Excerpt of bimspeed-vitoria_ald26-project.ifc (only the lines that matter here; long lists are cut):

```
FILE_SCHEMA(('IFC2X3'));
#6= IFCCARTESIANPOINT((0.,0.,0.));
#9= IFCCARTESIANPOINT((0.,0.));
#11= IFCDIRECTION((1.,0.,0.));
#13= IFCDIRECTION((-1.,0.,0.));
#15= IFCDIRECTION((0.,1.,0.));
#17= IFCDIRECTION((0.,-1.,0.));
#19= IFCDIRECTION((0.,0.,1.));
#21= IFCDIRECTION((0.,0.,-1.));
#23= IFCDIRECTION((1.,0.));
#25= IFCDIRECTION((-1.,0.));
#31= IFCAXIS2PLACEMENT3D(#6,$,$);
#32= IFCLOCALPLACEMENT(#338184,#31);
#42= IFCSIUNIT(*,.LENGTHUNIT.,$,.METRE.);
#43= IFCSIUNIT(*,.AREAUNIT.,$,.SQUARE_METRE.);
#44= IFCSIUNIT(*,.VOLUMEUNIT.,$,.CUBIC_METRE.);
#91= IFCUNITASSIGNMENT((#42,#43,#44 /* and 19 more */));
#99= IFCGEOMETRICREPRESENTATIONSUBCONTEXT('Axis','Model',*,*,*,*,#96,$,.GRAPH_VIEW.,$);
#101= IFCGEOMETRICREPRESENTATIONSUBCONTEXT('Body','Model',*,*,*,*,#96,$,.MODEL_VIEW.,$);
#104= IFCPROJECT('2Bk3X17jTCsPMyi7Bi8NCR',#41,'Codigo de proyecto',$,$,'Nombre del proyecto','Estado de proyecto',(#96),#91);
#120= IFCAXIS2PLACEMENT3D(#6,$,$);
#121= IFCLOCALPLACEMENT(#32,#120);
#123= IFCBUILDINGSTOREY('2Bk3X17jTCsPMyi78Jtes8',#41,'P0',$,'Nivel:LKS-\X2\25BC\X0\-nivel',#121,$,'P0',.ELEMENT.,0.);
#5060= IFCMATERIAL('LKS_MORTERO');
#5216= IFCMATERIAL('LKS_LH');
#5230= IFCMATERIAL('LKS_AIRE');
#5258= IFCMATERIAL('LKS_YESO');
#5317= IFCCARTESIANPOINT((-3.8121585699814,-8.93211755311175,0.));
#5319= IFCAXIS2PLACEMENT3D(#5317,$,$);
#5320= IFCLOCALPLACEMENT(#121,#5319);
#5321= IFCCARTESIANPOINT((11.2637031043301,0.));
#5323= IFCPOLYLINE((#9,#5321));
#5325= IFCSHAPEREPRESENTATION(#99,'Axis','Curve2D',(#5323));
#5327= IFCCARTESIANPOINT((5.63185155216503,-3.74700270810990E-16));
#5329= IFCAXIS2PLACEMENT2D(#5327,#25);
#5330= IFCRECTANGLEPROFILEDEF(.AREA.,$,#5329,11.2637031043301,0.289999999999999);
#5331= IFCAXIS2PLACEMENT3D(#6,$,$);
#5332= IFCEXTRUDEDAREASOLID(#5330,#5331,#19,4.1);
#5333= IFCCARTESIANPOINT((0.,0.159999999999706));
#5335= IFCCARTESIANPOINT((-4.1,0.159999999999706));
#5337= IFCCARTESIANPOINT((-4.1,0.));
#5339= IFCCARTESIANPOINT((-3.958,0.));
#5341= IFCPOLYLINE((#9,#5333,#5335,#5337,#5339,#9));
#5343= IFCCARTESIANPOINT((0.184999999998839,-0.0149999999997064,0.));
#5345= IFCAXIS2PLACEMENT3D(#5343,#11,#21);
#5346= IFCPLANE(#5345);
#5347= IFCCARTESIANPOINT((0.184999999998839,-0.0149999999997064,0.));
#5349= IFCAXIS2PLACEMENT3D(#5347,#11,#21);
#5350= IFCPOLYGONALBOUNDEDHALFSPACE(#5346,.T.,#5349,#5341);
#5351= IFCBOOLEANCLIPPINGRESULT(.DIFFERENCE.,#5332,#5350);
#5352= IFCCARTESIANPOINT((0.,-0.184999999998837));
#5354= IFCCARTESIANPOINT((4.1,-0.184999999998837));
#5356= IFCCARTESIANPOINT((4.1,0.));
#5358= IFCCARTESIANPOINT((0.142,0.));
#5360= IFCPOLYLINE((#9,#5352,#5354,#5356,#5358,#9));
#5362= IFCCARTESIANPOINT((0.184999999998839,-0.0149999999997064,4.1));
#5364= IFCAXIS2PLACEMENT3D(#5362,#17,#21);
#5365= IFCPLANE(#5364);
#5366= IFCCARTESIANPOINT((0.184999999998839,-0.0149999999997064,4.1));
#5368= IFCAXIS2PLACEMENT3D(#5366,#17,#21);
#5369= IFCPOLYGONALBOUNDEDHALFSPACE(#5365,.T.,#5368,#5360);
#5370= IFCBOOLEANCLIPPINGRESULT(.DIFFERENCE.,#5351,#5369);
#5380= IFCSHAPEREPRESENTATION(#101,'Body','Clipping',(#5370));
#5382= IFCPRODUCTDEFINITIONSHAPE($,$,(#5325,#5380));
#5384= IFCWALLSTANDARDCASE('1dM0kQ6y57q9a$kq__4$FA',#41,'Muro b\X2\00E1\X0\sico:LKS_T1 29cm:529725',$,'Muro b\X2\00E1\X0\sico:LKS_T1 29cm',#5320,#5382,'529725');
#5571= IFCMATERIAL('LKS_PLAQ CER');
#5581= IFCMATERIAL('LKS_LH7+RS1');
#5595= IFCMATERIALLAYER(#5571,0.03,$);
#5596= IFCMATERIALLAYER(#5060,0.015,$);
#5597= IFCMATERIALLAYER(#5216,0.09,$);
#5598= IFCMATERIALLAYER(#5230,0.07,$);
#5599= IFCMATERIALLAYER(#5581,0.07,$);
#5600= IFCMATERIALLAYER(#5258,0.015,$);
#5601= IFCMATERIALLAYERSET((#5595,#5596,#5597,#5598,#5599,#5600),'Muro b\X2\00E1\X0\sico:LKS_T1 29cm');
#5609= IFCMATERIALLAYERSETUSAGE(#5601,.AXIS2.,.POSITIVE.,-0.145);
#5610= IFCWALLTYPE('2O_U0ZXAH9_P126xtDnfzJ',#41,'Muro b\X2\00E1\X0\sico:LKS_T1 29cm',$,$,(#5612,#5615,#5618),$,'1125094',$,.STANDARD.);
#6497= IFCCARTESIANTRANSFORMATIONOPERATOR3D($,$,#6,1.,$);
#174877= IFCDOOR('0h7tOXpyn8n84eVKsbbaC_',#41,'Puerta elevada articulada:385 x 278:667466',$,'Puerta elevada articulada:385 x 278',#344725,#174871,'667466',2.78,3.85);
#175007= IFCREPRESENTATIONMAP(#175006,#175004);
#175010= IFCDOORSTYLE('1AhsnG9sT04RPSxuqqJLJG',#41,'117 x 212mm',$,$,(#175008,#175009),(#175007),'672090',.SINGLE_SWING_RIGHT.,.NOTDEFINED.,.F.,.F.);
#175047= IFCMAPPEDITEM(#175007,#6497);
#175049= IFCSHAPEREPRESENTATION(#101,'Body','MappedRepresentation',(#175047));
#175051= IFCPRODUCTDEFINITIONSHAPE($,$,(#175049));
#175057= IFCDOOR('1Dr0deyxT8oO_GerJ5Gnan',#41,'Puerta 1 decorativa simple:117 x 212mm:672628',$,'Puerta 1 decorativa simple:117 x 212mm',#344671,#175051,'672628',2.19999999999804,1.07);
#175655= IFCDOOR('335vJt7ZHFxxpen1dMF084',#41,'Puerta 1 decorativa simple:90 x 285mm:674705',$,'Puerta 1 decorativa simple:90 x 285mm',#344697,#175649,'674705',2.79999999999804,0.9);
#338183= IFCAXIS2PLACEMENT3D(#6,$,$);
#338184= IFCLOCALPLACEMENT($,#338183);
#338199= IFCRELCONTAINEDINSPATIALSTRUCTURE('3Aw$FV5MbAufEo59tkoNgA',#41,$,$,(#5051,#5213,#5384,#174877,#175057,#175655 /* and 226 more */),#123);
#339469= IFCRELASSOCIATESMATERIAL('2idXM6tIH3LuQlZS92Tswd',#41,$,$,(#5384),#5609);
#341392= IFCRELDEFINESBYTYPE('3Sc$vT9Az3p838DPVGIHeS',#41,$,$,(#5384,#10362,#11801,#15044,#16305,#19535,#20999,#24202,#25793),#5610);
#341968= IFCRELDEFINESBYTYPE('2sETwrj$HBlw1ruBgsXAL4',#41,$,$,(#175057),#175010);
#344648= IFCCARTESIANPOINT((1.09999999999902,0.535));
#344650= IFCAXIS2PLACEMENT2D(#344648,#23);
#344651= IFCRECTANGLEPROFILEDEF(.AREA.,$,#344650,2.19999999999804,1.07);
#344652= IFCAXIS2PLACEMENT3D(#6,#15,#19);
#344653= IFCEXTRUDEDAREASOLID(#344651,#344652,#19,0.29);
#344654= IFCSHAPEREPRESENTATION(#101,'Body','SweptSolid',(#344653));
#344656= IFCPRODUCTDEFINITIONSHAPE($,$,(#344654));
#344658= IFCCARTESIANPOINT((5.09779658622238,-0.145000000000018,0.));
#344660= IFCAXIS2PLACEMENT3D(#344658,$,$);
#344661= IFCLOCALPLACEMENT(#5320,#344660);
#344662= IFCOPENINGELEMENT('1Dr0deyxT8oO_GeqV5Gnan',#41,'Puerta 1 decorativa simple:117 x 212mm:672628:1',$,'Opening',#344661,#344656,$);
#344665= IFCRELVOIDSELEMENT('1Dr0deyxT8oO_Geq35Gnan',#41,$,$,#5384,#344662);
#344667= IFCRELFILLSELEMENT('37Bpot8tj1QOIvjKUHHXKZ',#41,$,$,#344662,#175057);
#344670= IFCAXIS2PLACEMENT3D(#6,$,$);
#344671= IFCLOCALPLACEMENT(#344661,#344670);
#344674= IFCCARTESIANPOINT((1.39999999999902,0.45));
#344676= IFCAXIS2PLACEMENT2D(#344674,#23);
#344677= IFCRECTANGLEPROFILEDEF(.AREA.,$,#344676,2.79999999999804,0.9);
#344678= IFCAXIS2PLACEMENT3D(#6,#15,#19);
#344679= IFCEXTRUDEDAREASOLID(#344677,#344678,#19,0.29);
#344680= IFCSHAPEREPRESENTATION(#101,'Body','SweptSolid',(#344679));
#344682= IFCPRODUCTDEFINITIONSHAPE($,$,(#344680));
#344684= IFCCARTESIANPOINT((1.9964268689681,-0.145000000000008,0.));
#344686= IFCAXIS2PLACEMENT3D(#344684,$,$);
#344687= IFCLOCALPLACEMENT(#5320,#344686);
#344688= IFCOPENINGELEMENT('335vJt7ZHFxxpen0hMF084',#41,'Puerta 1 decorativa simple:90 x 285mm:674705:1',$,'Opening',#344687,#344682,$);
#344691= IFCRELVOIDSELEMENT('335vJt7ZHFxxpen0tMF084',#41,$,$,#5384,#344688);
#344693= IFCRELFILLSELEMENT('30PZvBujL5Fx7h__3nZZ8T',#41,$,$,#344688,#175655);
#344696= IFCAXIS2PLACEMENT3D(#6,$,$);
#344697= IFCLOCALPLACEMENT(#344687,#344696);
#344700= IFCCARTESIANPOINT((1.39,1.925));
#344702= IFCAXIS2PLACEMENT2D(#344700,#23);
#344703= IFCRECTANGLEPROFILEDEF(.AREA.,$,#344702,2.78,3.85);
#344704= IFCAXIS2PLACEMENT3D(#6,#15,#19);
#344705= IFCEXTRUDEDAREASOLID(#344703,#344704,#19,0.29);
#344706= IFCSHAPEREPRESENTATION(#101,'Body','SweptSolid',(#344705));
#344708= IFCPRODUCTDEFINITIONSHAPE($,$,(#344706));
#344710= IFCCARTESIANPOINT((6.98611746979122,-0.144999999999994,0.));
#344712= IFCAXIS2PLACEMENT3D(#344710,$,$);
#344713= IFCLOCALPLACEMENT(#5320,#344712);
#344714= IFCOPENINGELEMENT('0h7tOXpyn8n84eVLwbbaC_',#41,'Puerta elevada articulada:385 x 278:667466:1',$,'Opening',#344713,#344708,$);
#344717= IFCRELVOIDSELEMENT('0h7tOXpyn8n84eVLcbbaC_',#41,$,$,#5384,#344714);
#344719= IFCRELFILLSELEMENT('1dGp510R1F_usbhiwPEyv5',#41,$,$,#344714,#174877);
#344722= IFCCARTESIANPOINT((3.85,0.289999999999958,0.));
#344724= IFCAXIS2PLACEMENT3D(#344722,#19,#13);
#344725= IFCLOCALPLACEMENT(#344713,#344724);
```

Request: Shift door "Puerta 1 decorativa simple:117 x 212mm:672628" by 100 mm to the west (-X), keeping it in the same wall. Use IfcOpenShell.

```python
import ifcopenshell
import ifcopenshell.api.geometry
import ifcopenshell.util.placement
import ifcopenshell.util.unit

model = ifcopenshell.open("bimspeed-vitoria_ald26-project.ifc")
unit_scale = ifcopenshell.util.unit.calculate_unit_scale(model)

door = model.by_guid("1Dr0deyxT8oO_GerJ5Gnan")
opening = door.FillsVoids[0].RelatingOpeningElement
wall = opening.VoidsElements[0].RelatingBuildingElement

wall_matrix = ifcopenshell.util.placement.get_local_placement(wall.ObjectPlacement)
shift = wall_matrix[:3, 0] * -0.1 / unit_scale
before = ifcopenshell.util.placement.get_local_placement(door.ObjectPlacement)[:3, 3].copy()

# The door is placed relative to its opening, so it follows when the opening moves.
matrix = ifcopenshell.util.placement.get_local_placement(opening.ObjectPlacement)
matrix[:3, 3] += shift
ifcopenshell.api.geometry.edit_object_placement(
    model, product=opening, matrix=matrix, is_si=False, should_transform_children=True
)

after = ifcopenshell.util.placement.get_local_placement(door.ObjectPlacement)[:3, 3]
print("door moved by", (after - before).round(3) + 0.0)

model.write("bimspeed-vitoria_ald26-project_edited.ifc")
```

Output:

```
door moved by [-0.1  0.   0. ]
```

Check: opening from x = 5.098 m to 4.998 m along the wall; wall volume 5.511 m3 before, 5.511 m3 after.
